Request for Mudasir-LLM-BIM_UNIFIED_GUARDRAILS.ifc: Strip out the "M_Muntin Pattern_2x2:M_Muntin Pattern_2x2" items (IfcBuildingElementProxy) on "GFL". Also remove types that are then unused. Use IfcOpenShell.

First a look at what the model holds.

```python
import ifcopenshell
import ifcopenshell.util.element

model = ifcopenshell.open("Mudasir-LLM-BIM_UNIFIED_GUARDRAILS.ifc")
print(model.schema)
storey = next(s for s in model.by_type("IfcBuildingStorey") if s.Name == "GFL")
proxies = [e for e in ifcopenshell.util.element.get_decomposition(storey) if e.is_a("IfcBuildingElementProxy")]
seen = {}
for e in proxies:
    element_type = ifcopenshell.util.element.get_type(e)
    name = element_type.Name if element_type not in (None, e) else None
    seen[name] = seen.get(name, 0) + 1
for name, count in sorted(seen.items(), key=str):
    print(count, "x", name)
```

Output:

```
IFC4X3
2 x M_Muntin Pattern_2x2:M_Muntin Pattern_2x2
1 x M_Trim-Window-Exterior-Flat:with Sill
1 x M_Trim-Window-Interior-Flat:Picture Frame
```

```python
import ifcopenshell
import ifcopenshell.api.root
import ifcopenshell.util.element

model = ifcopenshell.open("Mudasir-LLM-BIM_UNIFIED_GUARDRAILS.ifc")

storey = next(s for s in model.by_type("IfcBuildingStorey") if s.Name == "GFL")
proxies = [e for e in ifcopenshell.util.element.get_decomposition(storey) if e.is_a("IfcBuildingElementProxy")]
targets = [e for e in proxies if (t := ifcopenshell.util.element.get_type(e)) not in (None, e) and t.Name == "M_Muntin Pattern_2x2:M_Muntin Pattern_2x2"]
types = {ifcopenshell.util.element.get_type(e) for e in targets} - {None, *targets}

for e in targets:
    ifcopenshell.api.root.remove_product(model, product=e)
print(len(targets), "removed")

unused = [t for t in types if not ifcopenshell.util.element.get_types(t)]
for t in unused:
    ifcopenshell.api.root.remove_product(model, product=t)
print(len(unused), "unused types removed")

model.write("Mudasir-LLM-BIM_UNIFIED_GUARDRAILS_rev.ifc")
```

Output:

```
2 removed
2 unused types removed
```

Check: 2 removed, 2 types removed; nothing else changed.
